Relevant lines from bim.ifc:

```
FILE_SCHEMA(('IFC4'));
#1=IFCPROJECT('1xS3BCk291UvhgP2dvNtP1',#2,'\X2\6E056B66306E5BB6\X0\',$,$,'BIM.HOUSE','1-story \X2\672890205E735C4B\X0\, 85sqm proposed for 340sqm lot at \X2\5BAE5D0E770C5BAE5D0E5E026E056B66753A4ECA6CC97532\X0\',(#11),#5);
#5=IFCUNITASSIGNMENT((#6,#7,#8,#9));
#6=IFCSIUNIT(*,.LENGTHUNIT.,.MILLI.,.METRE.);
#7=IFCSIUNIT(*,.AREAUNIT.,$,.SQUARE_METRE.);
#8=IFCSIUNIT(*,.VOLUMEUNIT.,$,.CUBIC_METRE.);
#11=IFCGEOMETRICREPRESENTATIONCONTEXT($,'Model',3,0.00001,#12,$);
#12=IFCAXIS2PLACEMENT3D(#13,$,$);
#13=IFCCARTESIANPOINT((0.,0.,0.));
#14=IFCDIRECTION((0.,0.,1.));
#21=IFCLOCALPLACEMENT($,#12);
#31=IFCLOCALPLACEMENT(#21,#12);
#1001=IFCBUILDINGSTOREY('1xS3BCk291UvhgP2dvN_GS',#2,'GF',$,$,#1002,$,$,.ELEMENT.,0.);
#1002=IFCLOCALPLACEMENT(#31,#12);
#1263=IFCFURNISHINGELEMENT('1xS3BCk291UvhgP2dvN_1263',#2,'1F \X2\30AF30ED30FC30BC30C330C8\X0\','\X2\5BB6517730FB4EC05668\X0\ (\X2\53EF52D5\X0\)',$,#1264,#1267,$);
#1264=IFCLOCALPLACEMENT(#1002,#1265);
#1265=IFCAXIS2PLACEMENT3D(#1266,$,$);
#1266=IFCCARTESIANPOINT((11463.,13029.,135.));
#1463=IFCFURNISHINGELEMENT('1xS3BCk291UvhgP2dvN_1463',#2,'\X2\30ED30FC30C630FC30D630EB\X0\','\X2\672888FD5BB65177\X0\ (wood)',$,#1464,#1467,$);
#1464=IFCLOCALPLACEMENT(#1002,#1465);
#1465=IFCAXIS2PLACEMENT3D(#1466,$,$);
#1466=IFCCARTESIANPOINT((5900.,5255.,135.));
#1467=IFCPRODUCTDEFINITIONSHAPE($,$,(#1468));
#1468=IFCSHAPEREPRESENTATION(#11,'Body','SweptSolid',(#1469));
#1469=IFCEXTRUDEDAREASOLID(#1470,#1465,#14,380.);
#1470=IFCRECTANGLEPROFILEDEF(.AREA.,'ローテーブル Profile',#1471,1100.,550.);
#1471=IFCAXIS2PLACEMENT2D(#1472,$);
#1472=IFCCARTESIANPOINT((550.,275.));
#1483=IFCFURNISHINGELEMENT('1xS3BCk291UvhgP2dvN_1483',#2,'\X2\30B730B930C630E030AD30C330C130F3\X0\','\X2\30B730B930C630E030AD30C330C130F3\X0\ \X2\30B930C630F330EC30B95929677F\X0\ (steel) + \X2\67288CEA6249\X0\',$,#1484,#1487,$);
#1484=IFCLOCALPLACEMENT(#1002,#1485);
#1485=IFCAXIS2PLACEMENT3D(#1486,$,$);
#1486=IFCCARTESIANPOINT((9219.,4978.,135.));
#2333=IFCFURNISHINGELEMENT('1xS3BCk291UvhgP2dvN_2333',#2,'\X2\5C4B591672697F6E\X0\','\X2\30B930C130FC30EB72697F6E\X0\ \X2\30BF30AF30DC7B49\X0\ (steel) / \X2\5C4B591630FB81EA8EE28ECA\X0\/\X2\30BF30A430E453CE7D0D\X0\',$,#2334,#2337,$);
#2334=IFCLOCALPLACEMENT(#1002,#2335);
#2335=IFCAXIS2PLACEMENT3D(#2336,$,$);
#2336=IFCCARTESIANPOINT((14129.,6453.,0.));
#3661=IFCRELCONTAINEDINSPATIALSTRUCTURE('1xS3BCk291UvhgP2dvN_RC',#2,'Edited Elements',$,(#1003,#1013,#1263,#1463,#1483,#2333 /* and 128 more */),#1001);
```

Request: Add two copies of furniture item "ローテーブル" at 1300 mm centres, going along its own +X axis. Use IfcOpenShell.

```python
import ifcopenshell
import ifcopenshell.api.geometry
import ifcopenshell.api.root
import ifcopenshell.util.element
import ifcopenshell.util.placement

model = ifcopenshell.open("bim.ifc")


def reuse_history(source, copy):
    """copy_class also copies each property set's owner history, people and application; keep the originals."""
    for rel in copy.IsDefinedBy:
        if rel.is_a("IfcRelDefinesByProperties") and (history := rel.RelatingPropertyDefinition.OwnerHistory):
            rel.RelatingPropertyDefinition.OwnerHistory = source.OwnerHistory
            ifcopenshell.util.element.remove_deep2(model, history)


source = model.by_guid("1xS3BCk291UvhgP2dvN_1463")
base = ifcopenshell.util.placement.get_local_placement(source.ObjectPlacement)
step = base[:3, 0] * 1300.0

for i in range(1, 3):
    copy = ifcopenshell.api.root.copy_class(model, product=source)
    copy.Representation = ifcopenshell.util.element.copy_deep(
        model, source.Representation, exclude=["IfcGeometricRepresentationContext", "IfcRepresentationMap"]
    )
    reuse_history(source, copy)
    matrix = base.copy()
    matrix[:3, 3] += i * step
    print("added at", matrix[:3, 3].round(3) + 0.0)
    ifcopenshell.api.geometry.edit_object_placement(model, product=copy, matrix=matrix, is_si=False)

model.write("bim_rev.ifc")
```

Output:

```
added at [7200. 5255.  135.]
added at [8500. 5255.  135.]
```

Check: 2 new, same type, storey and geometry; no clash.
